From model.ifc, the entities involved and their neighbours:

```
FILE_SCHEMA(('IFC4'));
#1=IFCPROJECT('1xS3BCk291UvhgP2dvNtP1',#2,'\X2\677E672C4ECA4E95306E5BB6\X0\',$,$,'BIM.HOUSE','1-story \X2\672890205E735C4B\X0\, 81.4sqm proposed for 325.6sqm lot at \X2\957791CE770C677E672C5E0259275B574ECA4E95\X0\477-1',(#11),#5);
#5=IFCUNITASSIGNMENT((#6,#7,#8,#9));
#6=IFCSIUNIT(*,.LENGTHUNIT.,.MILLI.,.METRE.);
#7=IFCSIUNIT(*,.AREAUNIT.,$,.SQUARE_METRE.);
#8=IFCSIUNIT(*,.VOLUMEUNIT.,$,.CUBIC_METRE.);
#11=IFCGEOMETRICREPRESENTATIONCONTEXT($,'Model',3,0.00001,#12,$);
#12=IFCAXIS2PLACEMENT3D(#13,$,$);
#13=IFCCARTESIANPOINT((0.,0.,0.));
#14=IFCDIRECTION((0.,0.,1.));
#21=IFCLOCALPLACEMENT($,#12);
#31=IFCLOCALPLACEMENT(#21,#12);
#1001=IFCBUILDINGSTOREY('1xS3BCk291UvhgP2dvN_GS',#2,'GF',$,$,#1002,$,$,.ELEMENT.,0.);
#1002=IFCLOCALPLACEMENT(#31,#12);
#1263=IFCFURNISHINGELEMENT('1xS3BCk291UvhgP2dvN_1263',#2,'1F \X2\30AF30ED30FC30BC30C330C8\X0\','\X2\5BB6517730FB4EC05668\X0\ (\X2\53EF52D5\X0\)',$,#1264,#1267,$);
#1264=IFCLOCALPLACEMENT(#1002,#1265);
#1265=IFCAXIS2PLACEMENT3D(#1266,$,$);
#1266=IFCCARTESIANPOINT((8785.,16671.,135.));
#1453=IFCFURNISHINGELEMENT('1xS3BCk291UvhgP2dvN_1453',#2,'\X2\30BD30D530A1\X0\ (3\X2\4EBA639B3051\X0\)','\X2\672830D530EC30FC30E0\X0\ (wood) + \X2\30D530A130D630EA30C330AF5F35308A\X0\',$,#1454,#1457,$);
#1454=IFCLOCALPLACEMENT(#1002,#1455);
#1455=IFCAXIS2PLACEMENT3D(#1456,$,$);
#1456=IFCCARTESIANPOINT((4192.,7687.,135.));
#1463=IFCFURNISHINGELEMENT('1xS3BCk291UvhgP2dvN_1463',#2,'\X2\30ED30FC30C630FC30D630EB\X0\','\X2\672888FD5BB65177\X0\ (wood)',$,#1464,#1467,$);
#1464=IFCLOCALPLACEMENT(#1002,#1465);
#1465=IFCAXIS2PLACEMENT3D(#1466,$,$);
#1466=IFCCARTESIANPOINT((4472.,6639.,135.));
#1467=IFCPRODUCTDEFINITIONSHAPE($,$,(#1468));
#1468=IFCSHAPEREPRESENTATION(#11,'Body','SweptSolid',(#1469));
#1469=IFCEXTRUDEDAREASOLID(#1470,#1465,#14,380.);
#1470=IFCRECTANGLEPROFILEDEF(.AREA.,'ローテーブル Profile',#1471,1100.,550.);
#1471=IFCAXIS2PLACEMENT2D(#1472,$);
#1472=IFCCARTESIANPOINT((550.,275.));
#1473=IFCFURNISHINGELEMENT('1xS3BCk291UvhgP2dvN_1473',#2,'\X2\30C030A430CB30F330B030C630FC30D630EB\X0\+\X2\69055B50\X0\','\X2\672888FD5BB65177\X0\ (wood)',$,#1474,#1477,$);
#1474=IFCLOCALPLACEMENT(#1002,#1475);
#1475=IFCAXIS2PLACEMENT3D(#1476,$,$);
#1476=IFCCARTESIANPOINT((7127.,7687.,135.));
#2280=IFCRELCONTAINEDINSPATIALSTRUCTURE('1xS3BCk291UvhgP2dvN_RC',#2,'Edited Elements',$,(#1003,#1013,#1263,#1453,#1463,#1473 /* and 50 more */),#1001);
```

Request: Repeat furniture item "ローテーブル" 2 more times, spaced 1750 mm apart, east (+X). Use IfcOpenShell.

```python
import numpy as np
import ifcopenshell
import ifcopenshell.api.geometry
import ifcopenshell.api.root
import ifcopenshell.util.element
import ifcopenshell.util.placement

model = ifcopenshell.open("model.ifc")


def reuse_history(source, copy):
    """copy_class also copies each property set's owner history, people and application; keep the originals."""
    for rel in copy.IsDefinedBy:
        if rel.is_a("IfcRelDefinesByProperties") and (history := rel.RelatingPropertyDefinition.OwnerHistory):
            rel.RelatingPropertyDefinition.OwnerHistory = source.OwnerHistory
            ifcopenshell.util.element.remove_deep2(model, history)


source = model.by_guid("1xS3BCk291UvhgP2dvN_1463")
base = ifcopenshell.util.placement.get_local_placement(source.ObjectPlacement)
step = np.array([1.0, 0.0, 0.0]) * 1750.0

for i in range(1, 3):
    copy = ifcopenshell.api.root.copy_class(model, product=source)
    copy.Representation = ifcopenshell.util.element.copy_deep(
        model, source.Representation, exclude=["IfcGeometricRepresentationContext", "IfcRepresentationMap"]
    )
    reuse_history(source, copy)
    matrix = base.copy()
    matrix[:3, 3] += i * step
    print("added at", matrix[:3, 3].round(3) + 0.0)
    ifcopenshell.api.geometry.edit_object_placement(model, product=copy, matrix=matrix, is_si=False)

model.write("model_updated.ifc")
```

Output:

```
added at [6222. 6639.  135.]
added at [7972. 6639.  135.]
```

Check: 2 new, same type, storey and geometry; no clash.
